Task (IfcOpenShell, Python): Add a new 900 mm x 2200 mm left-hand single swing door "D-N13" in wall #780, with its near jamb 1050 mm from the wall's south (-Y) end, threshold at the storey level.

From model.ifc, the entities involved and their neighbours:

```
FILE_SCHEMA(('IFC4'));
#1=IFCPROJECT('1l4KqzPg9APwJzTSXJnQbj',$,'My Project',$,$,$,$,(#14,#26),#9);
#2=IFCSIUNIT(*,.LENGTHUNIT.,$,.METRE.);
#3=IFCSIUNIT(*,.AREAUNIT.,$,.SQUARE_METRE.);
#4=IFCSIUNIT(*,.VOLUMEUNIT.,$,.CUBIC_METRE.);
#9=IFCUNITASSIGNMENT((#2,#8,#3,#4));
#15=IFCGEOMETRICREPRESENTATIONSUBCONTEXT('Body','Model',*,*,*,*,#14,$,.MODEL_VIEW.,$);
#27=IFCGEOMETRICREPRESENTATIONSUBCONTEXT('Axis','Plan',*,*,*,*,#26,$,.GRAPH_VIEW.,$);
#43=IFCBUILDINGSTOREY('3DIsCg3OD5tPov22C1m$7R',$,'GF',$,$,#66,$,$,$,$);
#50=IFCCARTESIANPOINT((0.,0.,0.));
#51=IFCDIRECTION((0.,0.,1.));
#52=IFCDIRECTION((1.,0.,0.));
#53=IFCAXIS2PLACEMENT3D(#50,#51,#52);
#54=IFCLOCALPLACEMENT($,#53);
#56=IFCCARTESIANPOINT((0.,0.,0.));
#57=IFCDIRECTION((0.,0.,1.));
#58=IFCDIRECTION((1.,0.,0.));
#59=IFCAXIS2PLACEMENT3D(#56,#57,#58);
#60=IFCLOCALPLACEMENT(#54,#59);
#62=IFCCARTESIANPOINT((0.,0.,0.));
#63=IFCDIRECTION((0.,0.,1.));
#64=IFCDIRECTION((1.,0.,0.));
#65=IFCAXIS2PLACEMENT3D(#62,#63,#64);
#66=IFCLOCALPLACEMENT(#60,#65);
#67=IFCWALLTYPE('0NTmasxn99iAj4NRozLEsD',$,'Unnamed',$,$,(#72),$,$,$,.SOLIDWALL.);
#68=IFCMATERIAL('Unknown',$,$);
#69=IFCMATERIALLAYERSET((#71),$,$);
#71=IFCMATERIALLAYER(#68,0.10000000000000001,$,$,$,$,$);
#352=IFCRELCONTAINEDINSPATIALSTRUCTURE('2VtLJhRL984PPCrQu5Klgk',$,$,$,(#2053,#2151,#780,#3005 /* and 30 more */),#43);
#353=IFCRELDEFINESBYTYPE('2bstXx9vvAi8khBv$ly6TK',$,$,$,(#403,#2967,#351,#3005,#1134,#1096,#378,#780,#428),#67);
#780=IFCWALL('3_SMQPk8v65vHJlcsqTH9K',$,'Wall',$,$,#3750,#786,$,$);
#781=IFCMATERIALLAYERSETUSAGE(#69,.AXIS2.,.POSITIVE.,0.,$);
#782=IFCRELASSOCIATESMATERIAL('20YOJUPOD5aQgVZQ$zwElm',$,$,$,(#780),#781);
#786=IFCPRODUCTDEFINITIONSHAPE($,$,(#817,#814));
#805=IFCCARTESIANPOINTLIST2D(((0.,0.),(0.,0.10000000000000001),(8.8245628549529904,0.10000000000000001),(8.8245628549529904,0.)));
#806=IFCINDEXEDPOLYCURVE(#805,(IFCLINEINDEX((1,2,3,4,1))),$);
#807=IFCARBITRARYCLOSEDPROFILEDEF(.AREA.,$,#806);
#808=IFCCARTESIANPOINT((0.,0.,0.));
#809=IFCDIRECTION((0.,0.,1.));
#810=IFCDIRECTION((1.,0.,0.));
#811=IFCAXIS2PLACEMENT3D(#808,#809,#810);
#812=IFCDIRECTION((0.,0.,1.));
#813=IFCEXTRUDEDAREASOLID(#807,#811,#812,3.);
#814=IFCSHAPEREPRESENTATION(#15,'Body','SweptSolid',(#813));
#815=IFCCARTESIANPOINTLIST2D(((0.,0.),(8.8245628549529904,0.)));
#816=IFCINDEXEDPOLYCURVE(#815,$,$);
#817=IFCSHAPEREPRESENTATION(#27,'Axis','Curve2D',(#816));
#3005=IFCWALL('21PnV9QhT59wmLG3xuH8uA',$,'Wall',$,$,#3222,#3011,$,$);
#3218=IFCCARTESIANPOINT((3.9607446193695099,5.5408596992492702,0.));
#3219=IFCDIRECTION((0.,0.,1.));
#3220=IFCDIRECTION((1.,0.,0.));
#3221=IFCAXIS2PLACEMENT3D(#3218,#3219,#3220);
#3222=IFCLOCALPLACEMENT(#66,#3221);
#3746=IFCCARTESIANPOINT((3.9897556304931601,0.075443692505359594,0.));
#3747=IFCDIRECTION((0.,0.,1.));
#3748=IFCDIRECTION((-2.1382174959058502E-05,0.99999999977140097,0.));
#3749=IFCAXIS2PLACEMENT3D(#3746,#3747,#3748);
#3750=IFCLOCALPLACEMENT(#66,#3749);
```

```python
import numpy as np
import ifcopenshell
import ifcopenshell.api.feature
import ifcopenshell.api.geometry
import ifcopenshell.api.root
import ifcopenshell.api.spatial
import ifcopenshell.geom
import ifcopenshell.util.element
import ifcopenshell.util.placement
import ifcopenshell.util.representation
import ifcopenshell.util.shape
import ifcopenshell.util.unit

model = ifcopenshell.open("model.ifc")
unit_scale = ifcopenshell.util.unit.calculate_unit_scale(model)
settings = ifcopenshell.geom.settings()


def volume(element):
    """Net volume in cubic metres, openings subtracted."""
    shape = ifcopenshell.geom.create_shape(settings, element)
    return ifcopenshell.util.shape.get_volume(shape.geometry)


wall = model.by_id(780)
storey = ifcopenshell.util.element.get_container(wall, ifc_class="IfcBuildingStorey")
context = ifcopenshell.util.representation.get_context(model, "Model", "Body", "MODEL_VIEW")
before = volume(wall)

width, height, from_end, sill = 0.9, 2.2, 1.05, 0.0  # metres

# The wall runs along its own X axis, and the end named is its -X end.
wall_shape = ifcopenshell.geom.create_shape(settings, wall)
x, y, z = ifcopenshell.util.shape.get_vertices(wall_shape.geometry).T
start = x.min() + from_end
face, thickness = float(y.min()), float(y.max() - y.min())
wall_matrix = ifcopenshell.util.placement.get_local_placement(wall.ObjectPlacement)
level = ifcopenshell.util.placement.get_local_placement(storey.ObjectPlacement)[2, 3]


def in_wall(x, y):
    """Placement at x, y metres in the wall's axes, at sill height."""
    matrix = wall_matrix.copy()
    matrix[:, 3] = wall_matrix @ np.array([x / unit_scale, y / unit_scale, 0.0, 1.0])
    matrix[2, 3] = level + sill / unit_scale
    return matrix


# Opening: a box that overshoots both wall faces by 50 mm.
opening = ifcopenshell.api.root.create_entity(model, ifc_class="IfcOpeningElement", predefined_type="OPENING")
box = ifcopenshell.api.geometry.add_wall_representation(
    model, context=context, length=width, height=height, thickness=thickness + 0.1
)
ifcopenshell.api.geometry.assign_representation(model, product=opening, representation=box)
ifcopenshell.api.geometry.edit_object_placement(model, product=opening, matrix=in_wall(start, face - 0.05), is_si=False)
ifcopenshell.api.feature.add_feature(model, feature=opening, element=wall)

door = ifcopenshell.api.root.create_entity(model, ifc_class="IfcDoor", name="D-N13", predefined_type="DOOR")
door.OverallWidth, door.OverallHeight = width / unit_scale, height / unit_scale
door.OperationType = "SINGLE_SWING_LEFT"
body = ifcopenshell.api.geometry.add_door_representation(
    model,
    context=context,
    overall_width=door.OverallWidth,
    overall_height=door.OverallHeight,
    operation_type="SINGLE_SWING_LEFT",
    lining_properties={"LiningDepth": thickness / unit_scale, "ThresholdDepth": thickness / unit_scale},
)
ifcopenshell.api.geometry.assign_representation(model, product=door, representation=body)
ifcopenshell.api.spatial.assign_container(model, products=[door], relating_structure=storey)
ifcopenshell.api.feature.add_filling(model, opening=opening, element=door)

# The lining spans the wall, so the door starts at the wall face.
ifcopenshell.api.geometry.edit_object_placement(model, product=door, matrix=in_wall(start, face), is_si=False)

after = volume(wall)

print(f"wall volume {before:.3f} -> {after:.3f} m3")

model.write("model_updated.ifc")
```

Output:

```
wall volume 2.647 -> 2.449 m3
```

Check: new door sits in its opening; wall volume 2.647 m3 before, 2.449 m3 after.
